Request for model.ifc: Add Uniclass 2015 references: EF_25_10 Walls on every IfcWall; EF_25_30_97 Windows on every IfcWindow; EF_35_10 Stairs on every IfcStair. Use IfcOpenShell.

First a look at what the model holds.

```python
import ifcopenshell

model = ifcopenshell.open("model.ifc")
print(model.schema)
print("classifications:", [c.Name for c in model.by_type("IfcClassification")])
for ifc_class in ("IfcDoor", "IfcRoof", "IfcStair", "IfcWall", "IfcWindow"):
    print(ifc_class, len(model.by_type(ifc_class)))
```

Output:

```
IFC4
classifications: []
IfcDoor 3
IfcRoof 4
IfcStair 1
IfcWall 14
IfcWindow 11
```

```python
import ifcopenshell
import ifcopenshell.api.classification

model = ifcopenshell.open("model.ifc")

system = ifcopenshell.api.classification.add_classification(model, classification="Uniclass 2015")

codes = {
    "IfcWall": ("EF_25_10", "Walls"),
    "IfcWindow": ("EF_25_30_97", "Windows"),
    "IfcStair": ("EF_35_10", "Stairs"),
}
for ifc_class, (code, name) in codes.items():
    products = model.by_type(ifc_class)
    ifcopenshell.api.classification.add_reference(
        model, products=products, classification=system, identification=code, name=name
    )
    print(code, len(products))

model.write("model-out.ifc")
```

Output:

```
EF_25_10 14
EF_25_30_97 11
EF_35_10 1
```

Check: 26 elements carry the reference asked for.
